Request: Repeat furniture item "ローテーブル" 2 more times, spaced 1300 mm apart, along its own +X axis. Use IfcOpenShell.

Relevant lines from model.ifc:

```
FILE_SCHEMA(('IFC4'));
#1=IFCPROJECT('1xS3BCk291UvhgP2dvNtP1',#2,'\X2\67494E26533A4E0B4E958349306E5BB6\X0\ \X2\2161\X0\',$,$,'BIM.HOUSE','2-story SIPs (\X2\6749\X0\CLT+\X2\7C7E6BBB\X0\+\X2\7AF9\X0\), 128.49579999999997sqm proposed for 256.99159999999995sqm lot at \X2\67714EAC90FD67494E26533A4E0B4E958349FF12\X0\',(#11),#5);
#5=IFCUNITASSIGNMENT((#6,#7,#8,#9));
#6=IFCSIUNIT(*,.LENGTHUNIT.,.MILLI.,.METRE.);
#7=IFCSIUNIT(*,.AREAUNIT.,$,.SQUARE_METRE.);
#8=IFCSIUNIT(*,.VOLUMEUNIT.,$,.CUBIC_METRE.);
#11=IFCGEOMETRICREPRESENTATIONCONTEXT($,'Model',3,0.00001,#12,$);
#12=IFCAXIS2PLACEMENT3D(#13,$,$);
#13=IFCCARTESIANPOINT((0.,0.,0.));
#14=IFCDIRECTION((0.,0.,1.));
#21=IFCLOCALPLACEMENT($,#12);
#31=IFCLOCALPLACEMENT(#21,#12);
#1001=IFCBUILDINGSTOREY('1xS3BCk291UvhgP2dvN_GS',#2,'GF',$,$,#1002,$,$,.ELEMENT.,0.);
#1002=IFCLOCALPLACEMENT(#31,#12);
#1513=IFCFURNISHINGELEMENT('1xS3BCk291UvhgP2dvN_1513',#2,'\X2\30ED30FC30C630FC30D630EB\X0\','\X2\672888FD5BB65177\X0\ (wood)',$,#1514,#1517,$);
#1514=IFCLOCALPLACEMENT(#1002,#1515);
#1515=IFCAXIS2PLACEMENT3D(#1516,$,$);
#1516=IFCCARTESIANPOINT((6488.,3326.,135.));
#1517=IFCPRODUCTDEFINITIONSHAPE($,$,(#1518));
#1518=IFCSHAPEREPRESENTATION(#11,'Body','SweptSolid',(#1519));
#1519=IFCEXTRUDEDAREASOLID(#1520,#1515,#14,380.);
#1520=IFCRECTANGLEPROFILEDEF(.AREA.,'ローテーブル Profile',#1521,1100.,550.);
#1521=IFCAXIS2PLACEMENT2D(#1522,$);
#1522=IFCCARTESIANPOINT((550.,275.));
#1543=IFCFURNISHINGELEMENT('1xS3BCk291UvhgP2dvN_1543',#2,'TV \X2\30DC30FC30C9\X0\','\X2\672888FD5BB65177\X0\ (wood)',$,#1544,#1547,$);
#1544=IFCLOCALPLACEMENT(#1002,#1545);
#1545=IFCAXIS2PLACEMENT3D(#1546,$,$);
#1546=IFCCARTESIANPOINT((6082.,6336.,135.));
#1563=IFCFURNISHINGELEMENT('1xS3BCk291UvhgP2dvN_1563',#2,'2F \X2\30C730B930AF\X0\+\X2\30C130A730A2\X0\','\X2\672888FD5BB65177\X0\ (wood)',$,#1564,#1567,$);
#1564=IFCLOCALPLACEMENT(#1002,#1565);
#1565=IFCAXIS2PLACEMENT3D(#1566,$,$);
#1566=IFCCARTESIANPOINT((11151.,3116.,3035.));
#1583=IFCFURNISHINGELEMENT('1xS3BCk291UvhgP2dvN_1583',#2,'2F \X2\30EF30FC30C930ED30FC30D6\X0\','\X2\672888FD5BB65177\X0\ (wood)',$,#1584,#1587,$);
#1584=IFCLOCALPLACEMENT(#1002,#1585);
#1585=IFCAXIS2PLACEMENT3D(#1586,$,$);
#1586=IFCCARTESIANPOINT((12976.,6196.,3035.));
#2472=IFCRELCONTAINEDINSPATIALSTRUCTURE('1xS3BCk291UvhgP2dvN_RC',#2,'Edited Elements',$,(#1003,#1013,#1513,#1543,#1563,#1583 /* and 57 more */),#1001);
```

```python
import ifcopenshell
import ifcopenshell.api.geometry
import ifcopenshell.api.root
import ifcopenshell.util.element
import ifcopenshell.util.placement
import ifcopenshell.util.unit

model = ifcopenshell.open("model.ifc")
unit_scale = ifcopenshell.util.unit.calculate_unit_scale(model)


def reuse_history(source, copy):
    """copy_class also copies each property set's owner history, people and application; keep the originals."""
    for rel in copy.IsDefinedBy:
        if rel.is_a("IfcRelDefinesByProperties") and (history := rel.RelatingPropertyDefinition.OwnerHistory):
            rel.RelatingPropertyDefinition.OwnerHistory = source.OwnerHistory
            ifcopenshell.util.element.remove_deep2(model, history)


source = model.by_guid("1xS3BCk291UvhgP2dvN_1513")
base = ifcopenshell.util.placement.get_local_placement(source.ObjectPlacement)
step = base[:3, 0] * 1.3 / unit_scale

for i in range(1, 3):
    copy = ifcopenshell.api.root.copy_class(model, product=source)
    copy.Representation = ifcopenshell.util.element.copy_deep(
        model, source.Representation, exclude=["IfcGeometricRepresentationContext", "IfcRepresentationMap"]
    )
    reuse_history(source, copy)
    matrix = base.copy()
    matrix[:3, 3] += i * step
    print("added at", matrix[:3, 3].round(3) + 0.0)
    ifcopenshell.api.geometry.edit_object_placement(model, product=copy, matrix=matrix, is_si=False)

model.write("model_updated.ifc")
```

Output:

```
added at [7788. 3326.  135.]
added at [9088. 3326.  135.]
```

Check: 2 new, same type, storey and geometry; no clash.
